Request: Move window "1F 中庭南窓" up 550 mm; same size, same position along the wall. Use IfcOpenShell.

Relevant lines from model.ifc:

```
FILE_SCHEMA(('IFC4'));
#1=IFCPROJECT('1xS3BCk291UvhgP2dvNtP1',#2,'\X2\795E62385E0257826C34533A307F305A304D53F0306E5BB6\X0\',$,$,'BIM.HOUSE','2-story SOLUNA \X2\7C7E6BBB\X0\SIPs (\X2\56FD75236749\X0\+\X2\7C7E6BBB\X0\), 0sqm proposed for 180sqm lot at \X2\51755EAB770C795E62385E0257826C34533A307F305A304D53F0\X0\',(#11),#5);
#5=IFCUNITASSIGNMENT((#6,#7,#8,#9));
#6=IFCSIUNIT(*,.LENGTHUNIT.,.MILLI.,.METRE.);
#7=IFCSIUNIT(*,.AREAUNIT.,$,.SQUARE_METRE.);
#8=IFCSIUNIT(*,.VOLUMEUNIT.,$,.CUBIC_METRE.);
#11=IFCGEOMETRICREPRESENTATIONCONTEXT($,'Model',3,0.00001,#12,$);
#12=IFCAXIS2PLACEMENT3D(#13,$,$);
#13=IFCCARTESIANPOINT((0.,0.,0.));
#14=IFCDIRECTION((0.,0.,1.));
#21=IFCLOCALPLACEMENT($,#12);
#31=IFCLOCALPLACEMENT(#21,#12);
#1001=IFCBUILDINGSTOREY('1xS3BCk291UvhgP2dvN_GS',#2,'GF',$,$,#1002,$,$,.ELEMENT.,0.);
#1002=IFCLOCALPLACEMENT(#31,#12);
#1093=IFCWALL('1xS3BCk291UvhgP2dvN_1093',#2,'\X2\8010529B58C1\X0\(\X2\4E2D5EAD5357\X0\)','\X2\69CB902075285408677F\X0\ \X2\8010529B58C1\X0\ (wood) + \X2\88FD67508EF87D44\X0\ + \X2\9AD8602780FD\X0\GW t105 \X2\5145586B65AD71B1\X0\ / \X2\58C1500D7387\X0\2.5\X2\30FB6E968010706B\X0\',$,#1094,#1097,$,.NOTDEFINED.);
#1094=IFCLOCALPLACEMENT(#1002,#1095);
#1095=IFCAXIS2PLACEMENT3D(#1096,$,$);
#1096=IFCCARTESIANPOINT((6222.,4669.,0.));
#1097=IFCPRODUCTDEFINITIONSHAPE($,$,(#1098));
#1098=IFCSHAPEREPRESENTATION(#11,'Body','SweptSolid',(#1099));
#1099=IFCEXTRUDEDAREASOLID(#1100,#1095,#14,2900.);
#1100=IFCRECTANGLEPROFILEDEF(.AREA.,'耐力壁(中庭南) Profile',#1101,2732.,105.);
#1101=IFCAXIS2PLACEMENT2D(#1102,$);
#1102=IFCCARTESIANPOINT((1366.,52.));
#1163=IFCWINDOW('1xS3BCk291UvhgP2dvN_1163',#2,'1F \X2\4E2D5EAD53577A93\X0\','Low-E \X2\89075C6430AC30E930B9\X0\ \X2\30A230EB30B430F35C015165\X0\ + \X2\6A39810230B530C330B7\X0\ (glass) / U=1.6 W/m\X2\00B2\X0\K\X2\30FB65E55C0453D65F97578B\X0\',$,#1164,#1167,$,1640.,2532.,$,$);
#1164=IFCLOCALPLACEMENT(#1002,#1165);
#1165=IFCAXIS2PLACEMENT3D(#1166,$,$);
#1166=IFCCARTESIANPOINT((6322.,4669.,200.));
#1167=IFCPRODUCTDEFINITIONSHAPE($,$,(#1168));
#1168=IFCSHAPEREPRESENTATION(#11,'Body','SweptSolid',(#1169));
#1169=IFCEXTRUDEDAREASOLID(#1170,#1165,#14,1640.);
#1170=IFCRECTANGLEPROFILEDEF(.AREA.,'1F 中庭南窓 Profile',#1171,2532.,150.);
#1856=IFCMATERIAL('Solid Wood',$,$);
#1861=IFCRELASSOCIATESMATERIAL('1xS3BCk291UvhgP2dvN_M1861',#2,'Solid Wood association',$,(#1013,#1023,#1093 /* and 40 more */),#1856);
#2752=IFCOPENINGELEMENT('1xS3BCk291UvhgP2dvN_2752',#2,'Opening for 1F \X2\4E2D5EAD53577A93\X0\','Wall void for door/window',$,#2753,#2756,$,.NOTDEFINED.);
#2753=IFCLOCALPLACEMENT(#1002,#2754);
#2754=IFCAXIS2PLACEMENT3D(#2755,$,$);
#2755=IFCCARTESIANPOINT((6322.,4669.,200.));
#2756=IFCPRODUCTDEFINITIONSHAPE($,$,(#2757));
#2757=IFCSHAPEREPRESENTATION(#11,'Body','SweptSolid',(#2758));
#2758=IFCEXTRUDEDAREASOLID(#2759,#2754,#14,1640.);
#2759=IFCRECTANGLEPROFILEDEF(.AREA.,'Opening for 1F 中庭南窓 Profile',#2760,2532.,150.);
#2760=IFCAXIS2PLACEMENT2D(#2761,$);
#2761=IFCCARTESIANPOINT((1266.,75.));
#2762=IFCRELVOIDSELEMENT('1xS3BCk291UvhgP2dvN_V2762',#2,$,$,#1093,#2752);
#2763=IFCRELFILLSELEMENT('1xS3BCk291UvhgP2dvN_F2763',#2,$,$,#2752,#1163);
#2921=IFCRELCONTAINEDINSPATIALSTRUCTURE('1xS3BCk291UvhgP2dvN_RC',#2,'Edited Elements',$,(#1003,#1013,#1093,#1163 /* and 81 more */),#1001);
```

```python
import numpy as np
import ifcopenshell
import ifcopenshell.api.geometry
import ifcopenshell.util.placement
import ifcopenshell.util.unit

model = ifcopenshell.open("model.ifc")
unit_scale = ifcopenshell.util.unit.calculate_unit_scale(model)

window = model.by_id(1163)
opening = window.FillsVoids[0].RelatingOpeningElement
dz = 0.55 / unit_scale

shift = np.array([0.0, 0.0, dz])
# The window is not placed relative to its opening, so move both.
for product in (opening, window):
    matrix = ifcopenshell.util.placement.get_local_placement(product.ObjectPlacement)
    matrix[:3, 3] += shift
    ifcopenshell.api.geometry.edit_object_placement(model, product=product, matrix=matrix, is_si=False)

print(f"moved by {dz * unit_scale:+.3f} m")

model.write("model_updated.ifc")
```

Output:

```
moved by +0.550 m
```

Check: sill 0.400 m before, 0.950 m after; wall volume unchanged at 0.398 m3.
